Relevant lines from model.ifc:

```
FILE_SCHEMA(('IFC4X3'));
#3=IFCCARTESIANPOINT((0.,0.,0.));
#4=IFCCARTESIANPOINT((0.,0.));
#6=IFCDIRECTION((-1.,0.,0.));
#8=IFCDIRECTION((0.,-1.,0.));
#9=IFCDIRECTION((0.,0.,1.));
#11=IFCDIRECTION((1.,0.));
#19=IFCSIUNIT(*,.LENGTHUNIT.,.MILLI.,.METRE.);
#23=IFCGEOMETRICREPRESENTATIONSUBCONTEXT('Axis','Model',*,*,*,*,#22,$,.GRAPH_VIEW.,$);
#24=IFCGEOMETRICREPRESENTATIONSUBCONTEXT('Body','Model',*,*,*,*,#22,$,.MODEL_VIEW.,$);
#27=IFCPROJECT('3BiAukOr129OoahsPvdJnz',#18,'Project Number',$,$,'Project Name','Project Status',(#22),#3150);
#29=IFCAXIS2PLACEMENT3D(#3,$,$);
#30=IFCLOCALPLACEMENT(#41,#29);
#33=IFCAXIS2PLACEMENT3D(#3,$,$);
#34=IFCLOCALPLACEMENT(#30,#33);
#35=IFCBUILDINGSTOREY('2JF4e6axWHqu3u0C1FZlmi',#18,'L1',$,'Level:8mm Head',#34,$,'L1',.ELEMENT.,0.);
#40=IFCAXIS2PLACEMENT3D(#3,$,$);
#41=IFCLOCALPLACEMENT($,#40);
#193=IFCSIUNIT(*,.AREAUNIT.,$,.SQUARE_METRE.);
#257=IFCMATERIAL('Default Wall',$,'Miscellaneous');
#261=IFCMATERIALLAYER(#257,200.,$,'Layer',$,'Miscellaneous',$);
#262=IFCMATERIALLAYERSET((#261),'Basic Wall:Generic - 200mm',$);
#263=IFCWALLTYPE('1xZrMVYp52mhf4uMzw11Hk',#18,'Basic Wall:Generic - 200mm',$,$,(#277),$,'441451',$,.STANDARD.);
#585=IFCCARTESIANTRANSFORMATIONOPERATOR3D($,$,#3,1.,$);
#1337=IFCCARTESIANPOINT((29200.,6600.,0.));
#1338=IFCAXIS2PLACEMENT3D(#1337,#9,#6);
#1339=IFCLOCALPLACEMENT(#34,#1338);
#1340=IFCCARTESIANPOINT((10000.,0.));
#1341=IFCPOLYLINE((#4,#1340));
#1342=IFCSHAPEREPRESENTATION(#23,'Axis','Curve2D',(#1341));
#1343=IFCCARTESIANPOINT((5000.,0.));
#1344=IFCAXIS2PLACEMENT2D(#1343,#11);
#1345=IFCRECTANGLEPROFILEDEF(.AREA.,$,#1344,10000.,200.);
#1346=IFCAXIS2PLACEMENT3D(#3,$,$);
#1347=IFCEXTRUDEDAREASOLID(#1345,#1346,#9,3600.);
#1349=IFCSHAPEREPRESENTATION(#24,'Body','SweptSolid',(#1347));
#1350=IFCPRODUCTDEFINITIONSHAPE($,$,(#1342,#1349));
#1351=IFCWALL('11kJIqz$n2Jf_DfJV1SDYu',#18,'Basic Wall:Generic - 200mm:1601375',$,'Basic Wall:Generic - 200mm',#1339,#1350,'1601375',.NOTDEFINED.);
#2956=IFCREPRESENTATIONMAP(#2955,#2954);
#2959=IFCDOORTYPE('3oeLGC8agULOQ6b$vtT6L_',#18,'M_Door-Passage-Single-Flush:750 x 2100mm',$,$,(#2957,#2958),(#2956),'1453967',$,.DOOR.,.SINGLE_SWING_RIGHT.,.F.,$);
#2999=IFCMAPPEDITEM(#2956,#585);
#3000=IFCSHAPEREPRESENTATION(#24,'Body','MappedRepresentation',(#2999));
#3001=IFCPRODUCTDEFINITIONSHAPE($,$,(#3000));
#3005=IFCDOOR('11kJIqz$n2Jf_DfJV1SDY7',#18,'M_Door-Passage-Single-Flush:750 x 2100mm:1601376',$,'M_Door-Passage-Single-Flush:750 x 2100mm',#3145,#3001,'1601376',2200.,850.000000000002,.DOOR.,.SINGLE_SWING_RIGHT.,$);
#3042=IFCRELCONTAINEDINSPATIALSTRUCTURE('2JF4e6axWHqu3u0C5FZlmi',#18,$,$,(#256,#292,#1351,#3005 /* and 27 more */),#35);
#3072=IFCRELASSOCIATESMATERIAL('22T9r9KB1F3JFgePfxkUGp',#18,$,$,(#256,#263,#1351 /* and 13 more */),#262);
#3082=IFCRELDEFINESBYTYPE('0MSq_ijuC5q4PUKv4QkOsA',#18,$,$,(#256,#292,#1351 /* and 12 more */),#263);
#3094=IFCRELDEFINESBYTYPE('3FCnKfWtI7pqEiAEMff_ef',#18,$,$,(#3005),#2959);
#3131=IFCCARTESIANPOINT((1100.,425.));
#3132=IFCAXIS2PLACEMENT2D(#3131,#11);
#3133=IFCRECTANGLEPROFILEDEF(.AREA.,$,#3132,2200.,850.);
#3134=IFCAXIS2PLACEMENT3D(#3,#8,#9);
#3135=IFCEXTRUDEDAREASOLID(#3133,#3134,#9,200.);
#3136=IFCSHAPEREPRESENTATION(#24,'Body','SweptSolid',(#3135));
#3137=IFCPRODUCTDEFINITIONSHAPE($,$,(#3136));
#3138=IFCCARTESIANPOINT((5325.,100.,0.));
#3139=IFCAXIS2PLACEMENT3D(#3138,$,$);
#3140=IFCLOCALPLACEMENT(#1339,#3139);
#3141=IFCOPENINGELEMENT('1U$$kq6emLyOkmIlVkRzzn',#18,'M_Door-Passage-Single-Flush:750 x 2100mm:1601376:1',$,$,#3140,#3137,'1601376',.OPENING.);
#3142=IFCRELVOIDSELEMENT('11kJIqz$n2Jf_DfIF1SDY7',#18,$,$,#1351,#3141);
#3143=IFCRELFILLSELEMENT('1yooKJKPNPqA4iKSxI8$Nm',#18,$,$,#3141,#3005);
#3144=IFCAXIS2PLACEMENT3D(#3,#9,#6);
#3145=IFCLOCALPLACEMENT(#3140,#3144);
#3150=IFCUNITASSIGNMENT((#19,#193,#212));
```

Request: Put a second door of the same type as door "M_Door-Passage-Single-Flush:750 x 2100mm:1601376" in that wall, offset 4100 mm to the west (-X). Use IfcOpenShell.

```python
import ifcopenshell
import ifcopenshell.api.feature
import ifcopenshell.api.geometry
import ifcopenshell.api.root
import ifcopenshell.geom
import ifcopenshell.util.element
import ifcopenshell.util.placement
import ifcopenshell.util.shape
import ifcopenshell.util.unit

model = ifcopenshell.open("model.ifc")
unit_scale = ifcopenshell.util.unit.calculate_unit_scale(model)
settings = ifcopenshell.geom.settings()


def volume(element):
    """Net volume in cubic metres, openings subtracted."""
    shape = ifcopenshell.geom.create_shape(settings, element)
    return ifcopenshell.util.shape.get_volume(shape.geometry)


def reuse_history(source, copy):
    """copy_class also copies each property set's owner history, people and application; keep the originals."""
    for rel in copy.IsDefinedBy:
        if rel.is_a("IfcRelDefinesByProperties") and (history := rel.RelatingPropertyDefinition.OwnerHistory):
            rel.RelatingPropertyDefinition.OwnerHistory = source.OwnerHistory
            ifcopenshell.util.element.remove_deep2(model, history)


door = model.by_guid("11kJIqz$n2Jf_DfJV1SDY7")
opening = door.FillsVoids[0].RelatingOpeningElement
wall = opening.VoidsElements[0].RelatingBuildingElement
before = volume(wall)
shift = ifcopenshell.util.placement.get_local_placement(wall.ObjectPlacement)[:3, 0] * 4.1 / unit_scale

# copy_class copies the void relationship, type, container and properties, but no geometry.
new_opening = ifcopenshell.api.root.copy_class(model, product=opening)
new_opening.Representation = ifcopenshell.util.element.copy_deep(
    model, opening.Representation, exclude=["IfcGeometricRepresentationContext", "IfcRepresentationMap"]
)
new_opening.Name = "M_Door-Passage-Single-Flush:750 x 2100mm"
new_opening.Tag = None
new_door = ifcopenshell.api.root.copy_class(model, product=door)
new_door.Representation = ifcopenshell.util.element.copy_deep(
    model, door.Representation, exclude=["IfcGeometricRepresentationContext", "IfcRepresentationMap"]
)
new_door.Name = "M_Door-Passage-Single-Flush:750 x 2100mm"
new_door.Tag = None
reuse_history(door, new_door)
ifcopenshell.api.feature.add_filling(model, opening=new_opening, element=new_door)

for old, new in ((opening, new_opening), (door, new_door)):
    matrix = ifcopenshell.util.placement.get_local_placement(old.ObjectPlacement)
    matrix[:3, 3] += shift
    ifcopenshell.api.geometry.edit_object_placement(model, product=new, matrix=matrix, is_si=False)

after = volume(wall)

print(f"wall volume {before:.3f} -> {after:.3f} m3")

model.write("model-out.ifc")
```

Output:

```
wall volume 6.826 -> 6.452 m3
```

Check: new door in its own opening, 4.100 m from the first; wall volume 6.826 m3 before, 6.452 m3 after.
